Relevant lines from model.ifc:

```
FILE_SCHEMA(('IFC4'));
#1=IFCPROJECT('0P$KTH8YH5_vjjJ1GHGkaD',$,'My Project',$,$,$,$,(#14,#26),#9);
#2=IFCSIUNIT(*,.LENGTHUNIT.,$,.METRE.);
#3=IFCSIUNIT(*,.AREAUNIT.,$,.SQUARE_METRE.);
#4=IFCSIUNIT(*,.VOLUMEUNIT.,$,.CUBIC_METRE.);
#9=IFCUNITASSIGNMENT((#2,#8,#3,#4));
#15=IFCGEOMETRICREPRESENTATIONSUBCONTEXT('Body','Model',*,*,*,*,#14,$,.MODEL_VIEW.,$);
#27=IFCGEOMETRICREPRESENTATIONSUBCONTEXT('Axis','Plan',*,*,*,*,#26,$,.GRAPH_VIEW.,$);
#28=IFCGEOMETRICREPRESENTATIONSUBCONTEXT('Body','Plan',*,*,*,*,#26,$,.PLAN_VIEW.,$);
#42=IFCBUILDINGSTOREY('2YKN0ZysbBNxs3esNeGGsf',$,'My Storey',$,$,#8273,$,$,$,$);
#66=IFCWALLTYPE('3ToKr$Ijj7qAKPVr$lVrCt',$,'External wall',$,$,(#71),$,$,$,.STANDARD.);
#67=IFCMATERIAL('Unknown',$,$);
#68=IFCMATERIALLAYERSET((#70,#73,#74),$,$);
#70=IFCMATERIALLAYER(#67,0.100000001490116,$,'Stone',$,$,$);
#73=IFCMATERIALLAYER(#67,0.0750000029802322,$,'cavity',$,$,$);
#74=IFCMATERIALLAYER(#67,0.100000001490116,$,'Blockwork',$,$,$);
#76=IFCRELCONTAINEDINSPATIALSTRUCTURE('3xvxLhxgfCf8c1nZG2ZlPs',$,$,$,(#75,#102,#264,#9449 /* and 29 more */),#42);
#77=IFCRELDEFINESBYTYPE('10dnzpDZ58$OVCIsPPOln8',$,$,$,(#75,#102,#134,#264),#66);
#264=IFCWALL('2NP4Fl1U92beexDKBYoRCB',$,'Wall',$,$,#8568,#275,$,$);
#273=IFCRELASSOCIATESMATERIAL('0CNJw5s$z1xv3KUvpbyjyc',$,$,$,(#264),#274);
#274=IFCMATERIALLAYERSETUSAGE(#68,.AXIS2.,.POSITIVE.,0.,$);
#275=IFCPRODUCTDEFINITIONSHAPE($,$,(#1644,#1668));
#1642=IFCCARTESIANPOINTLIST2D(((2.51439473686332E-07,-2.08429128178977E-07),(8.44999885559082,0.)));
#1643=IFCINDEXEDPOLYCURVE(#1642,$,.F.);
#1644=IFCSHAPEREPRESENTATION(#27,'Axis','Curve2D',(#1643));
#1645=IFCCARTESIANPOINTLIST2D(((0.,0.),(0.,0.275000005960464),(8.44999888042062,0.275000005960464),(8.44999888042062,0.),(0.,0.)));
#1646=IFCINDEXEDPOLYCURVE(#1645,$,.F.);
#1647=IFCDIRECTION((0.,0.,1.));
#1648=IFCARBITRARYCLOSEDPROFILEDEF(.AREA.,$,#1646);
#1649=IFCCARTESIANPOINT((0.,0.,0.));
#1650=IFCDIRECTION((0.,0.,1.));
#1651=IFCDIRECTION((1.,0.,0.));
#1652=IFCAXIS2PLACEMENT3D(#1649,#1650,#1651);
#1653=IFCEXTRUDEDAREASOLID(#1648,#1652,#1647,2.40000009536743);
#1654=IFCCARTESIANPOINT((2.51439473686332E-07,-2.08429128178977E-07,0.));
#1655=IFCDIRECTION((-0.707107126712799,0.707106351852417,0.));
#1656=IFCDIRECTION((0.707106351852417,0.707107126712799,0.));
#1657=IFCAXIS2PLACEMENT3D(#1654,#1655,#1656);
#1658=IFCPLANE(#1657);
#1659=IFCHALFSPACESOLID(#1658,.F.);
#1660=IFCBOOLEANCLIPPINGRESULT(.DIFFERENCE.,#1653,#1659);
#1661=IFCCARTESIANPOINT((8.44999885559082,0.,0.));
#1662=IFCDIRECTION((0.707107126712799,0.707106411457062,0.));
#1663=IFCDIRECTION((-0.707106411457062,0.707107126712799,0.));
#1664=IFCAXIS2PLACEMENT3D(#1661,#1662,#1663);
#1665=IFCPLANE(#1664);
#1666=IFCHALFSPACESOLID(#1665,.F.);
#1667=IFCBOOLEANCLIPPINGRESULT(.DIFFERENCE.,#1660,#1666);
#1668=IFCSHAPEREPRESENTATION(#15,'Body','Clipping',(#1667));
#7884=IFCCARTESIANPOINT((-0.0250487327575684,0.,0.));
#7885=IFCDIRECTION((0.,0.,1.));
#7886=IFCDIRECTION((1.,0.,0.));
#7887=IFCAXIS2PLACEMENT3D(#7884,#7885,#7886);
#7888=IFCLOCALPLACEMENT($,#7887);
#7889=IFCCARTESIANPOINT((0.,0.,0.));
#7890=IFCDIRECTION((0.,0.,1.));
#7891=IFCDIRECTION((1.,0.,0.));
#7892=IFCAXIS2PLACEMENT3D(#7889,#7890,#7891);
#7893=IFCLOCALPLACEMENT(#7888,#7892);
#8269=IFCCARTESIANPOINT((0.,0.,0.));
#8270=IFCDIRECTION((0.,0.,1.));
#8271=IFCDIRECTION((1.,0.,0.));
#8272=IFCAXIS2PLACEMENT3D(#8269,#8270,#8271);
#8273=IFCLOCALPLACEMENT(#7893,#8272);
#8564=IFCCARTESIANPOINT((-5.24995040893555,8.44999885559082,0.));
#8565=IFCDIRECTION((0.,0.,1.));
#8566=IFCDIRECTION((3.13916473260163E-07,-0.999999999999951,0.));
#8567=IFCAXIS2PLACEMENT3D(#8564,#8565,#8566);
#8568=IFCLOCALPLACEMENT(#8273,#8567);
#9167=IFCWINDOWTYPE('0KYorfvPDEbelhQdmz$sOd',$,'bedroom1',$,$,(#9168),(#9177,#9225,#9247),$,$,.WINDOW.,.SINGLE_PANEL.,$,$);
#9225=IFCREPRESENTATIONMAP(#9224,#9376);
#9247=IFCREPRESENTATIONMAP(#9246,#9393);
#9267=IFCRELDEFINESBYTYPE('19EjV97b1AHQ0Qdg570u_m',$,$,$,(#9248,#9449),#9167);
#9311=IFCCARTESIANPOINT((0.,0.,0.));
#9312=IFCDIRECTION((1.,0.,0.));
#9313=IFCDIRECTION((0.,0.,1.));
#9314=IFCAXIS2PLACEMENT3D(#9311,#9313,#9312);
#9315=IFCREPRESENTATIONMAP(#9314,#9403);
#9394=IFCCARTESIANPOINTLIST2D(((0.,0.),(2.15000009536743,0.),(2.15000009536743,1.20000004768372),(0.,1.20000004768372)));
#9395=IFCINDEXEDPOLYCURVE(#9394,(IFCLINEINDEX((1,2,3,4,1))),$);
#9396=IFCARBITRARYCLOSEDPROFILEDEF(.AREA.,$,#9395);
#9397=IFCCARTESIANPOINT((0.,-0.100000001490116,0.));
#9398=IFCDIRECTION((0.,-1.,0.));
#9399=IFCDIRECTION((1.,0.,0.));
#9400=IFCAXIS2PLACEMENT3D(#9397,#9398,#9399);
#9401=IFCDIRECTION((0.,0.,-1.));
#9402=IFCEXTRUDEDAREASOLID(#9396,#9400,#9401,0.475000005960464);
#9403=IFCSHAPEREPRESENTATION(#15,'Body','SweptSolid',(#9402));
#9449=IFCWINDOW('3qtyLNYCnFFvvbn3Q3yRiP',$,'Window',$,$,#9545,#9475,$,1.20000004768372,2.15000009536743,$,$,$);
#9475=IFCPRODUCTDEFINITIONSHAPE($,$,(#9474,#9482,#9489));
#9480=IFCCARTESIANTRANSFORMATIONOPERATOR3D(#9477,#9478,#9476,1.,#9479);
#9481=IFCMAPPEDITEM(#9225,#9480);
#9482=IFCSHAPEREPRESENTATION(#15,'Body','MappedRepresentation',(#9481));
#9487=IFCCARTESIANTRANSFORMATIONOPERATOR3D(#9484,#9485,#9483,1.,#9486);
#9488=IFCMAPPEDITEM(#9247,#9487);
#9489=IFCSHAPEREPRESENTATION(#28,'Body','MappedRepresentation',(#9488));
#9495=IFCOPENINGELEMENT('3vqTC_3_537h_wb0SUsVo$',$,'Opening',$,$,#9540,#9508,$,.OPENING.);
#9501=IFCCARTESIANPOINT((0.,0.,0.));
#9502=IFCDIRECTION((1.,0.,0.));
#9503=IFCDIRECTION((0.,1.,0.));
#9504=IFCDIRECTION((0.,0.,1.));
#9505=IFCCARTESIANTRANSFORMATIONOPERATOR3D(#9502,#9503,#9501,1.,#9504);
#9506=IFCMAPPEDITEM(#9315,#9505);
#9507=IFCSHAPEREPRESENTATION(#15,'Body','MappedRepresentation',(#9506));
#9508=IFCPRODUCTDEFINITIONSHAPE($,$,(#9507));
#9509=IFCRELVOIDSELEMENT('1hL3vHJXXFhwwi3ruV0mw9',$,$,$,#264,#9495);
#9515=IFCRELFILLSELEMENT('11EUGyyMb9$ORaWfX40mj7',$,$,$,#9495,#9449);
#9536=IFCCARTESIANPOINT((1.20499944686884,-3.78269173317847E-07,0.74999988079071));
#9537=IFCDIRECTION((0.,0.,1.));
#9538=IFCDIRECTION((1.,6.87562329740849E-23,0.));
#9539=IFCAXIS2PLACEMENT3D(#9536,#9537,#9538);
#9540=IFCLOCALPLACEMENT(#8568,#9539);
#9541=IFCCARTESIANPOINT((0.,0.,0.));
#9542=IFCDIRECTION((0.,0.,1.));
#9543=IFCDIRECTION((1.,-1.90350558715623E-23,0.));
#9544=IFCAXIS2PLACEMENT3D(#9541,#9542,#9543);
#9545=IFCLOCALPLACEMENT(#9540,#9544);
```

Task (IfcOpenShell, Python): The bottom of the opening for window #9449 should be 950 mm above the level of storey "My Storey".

```python
import numpy as np
import ifcopenshell
import ifcopenshell.api.geometry
import ifcopenshell.geom
import ifcopenshell.util.element
import ifcopenshell.util.placement
import ifcopenshell.util.shape
import ifcopenshell.util.unit

model = ifcopenshell.open("model.ifc")
unit_scale = ifcopenshell.util.unit.calculate_unit_scale(model)

window = model.by_id(9449)
opening = window.FillsVoids[0].RelatingOpeningElement
storey = ifcopenshell.util.element.get_container(window, ifc_class="IfcBuildingStorey")
level = ifcopenshell.util.placement.get_local_placement(storey.ObjectPlacement)[2, 3]

# The opening's origin need not be at the sill, so measure its lowest point.
shape = ifcopenshell.geom.create_shape(ifcopenshell.geom.settings(), opening)
bottom = ifcopenshell.util.shape.get_shape_bottom_elevation(shape, shape.geometry) / unit_scale
dz = level + 0.95 / unit_scale - bottom

shift = np.array([0.0, 0.0, dz])
# The window is placed relative to its opening, so it follows when the opening moves.
matrix = ifcopenshell.util.placement.get_local_placement(opening.ObjectPlacement)
matrix[:3, 3] += shift
ifcopenshell.api.geometry.edit_object_placement(
    model, product=opening, matrix=matrix, is_si=False, should_transform_children=True
)

print(f"moved by {dz * unit_scale:+.3f} m")

model.write("model_edited.ifc")
```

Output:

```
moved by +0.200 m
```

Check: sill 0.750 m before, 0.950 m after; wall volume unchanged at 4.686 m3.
